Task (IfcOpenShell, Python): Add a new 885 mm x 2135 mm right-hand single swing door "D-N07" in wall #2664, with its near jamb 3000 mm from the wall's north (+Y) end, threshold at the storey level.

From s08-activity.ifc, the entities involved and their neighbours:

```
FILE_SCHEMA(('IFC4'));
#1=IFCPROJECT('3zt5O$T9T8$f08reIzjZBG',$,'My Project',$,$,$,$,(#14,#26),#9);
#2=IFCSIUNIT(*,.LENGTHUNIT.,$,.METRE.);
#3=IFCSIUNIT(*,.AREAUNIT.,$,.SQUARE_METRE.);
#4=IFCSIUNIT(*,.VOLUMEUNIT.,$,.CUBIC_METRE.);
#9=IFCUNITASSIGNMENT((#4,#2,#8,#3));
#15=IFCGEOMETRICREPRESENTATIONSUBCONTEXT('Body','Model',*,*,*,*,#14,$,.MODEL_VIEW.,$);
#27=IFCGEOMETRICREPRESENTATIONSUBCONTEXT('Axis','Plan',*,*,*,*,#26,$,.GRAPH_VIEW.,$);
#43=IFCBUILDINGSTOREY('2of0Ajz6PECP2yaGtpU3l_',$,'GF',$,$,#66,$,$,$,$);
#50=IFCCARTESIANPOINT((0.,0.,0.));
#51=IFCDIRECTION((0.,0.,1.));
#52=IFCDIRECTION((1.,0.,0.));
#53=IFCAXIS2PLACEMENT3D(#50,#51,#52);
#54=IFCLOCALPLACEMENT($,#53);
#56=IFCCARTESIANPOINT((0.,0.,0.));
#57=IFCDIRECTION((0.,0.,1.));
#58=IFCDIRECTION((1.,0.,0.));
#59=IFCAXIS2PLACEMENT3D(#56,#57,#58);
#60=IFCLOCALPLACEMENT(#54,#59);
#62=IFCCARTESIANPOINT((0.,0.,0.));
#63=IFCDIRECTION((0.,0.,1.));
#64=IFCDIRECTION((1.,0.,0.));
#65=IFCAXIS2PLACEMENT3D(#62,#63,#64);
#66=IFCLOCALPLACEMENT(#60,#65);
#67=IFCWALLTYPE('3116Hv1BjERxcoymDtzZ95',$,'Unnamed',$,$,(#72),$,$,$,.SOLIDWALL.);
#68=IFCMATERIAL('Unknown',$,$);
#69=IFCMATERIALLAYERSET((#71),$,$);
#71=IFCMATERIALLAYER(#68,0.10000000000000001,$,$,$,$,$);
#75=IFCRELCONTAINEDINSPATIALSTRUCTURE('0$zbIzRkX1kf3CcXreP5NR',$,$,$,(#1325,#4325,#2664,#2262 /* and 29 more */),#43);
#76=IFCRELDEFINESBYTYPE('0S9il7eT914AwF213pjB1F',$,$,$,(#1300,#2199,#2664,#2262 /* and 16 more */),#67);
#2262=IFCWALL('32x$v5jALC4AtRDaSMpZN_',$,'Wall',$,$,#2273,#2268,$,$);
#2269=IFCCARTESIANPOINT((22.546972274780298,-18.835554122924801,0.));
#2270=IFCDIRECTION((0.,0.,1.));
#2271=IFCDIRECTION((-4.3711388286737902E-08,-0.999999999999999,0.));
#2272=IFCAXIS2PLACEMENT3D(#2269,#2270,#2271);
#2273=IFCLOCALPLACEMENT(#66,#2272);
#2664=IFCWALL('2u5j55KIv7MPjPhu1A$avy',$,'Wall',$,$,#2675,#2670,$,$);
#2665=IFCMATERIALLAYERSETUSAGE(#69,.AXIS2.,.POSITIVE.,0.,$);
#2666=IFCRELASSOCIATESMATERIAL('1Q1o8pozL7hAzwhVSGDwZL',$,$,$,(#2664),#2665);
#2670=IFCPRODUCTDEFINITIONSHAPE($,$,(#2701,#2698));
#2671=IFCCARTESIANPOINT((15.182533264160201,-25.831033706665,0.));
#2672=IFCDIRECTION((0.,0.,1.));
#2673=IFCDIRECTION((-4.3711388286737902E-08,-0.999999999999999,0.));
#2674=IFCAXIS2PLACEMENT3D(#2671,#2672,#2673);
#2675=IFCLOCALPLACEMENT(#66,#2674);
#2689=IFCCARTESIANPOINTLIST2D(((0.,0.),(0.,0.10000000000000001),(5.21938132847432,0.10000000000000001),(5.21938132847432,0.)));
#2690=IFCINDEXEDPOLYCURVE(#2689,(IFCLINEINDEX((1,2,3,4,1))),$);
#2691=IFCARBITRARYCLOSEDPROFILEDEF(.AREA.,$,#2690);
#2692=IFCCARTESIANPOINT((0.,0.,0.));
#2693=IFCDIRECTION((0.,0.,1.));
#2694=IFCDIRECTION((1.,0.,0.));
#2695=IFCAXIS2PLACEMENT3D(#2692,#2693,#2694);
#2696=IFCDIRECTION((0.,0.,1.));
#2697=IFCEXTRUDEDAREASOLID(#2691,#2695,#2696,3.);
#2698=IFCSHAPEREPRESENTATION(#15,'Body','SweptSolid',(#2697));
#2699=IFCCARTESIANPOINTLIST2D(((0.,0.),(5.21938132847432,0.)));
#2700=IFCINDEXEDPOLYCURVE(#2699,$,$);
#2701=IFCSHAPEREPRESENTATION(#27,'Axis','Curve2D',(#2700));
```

```python
import numpy as np
import ifcopenshell
import ifcopenshell.api.feature
import ifcopenshell.api.geometry
import ifcopenshell.api.root
import ifcopenshell.api.spatial
import ifcopenshell.geom
import ifcopenshell.util.element
import ifcopenshell.util.placement
import ifcopenshell.util.representation
import ifcopenshell.util.shape
import ifcopenshell.util.unit

model = ifcopenshell.open("s08-activity.ifc")
unit_scale = ifcopenshell.util.unit.calculate_unit_scale(model)
settings = ifcopenshell.geom.settings()


def volume(element):
    """Net volume in cubic metres, openings subtracted."""
    shape = ifcopenshell.geom.create_shape(settings, element)
    return ifcopenshell.util.shape.get_volume(shape.geometry)


wall = model.by_guid("2u5j55KIv7MPjPhu1A$avy")
storey = ifcopenshell.util.element.get_container(wall, ifc_class="IfcBuildingStorey")
context = ifcopenshell.util.representation.get_context(model, "Model", "Body", "MODEL_VIEW")
before = volume(wall)

width, height, from_end, sill = 0.885, 2.135, 3, 0.0  # metres

# The wall runs along its own X axis, and the end named is its -X end.
wall_shape = ifcopenshell.geom.create_shape(settings, wall)
x, y, z = ifcopenshell.util.shape.get_vertices(wall_shape.geometry).T
start = x.min() + from_end
face, thickness = float(y.min()), float(y.max() - y.min())
wall_matrix = ifcopenshell.util.placement.get_local_placement(wall.ObjectPlacement)
level = ifcopenshell.util.placement.get_local_placement(storey.ObjectPlacement)[2, 3]


def in_wall(x, y):
    """Placement at x, y metres in the wall's axes, at sill height."""
    matrix = wall_matrix.copy()
    matrix[:, 3] = wall_matrix @ np.array([x / unit_scale, y / unit_scale, 0.0, 1.0])
    matrix[2, 3] = level + sill / unit_scale
    return matrix


# Opening: a box that overshoots both wall faces by 50 mm.
opening = ifcopenshell.api.root.create_entity(model, ifc_class="IfcOpeningElement", predefined_type="OPENING")
box = ifcopenshell.api.geometry.add_wall_representation(
    model, context=context, length=width, height=height, thickness=thickness + 0.1
)
ifcopenshell.api.geometry.assign_representation(model, product=opening, representation=box)
ifcopenshell.api.geometry.edit_object_placement(model, product=opening, matrix=in_wall(start, face - 0.05), is_si=False)
ifcopenshell.api.feature.add_feature(model, feature=opening, element=wall)

door = ifcopenshell.api.root.create_entity(model, ifc_class="IfcDoor", name="D-N07", predefined_type="DOOR")
door.OverallWidth, door.OverallHeight = width / unit_scale, height / unit_scale
door.OperationType = "SINGLE_SWING_RIGHT"
body = ifcopenshell.api.geometry.add_door_representation(
    model,
    context=context,
    overall_width=door.OverallWidth,
    overall_height=door.OverallHeight,
    operation_type="SINGLE_SWING_RIGHT",
    lining_properties={"LiningDepth": thickness / unit_scale, "ThresholdDepth": thickness / unit_scale},
)
ifcopenshell.api.geometry.assign_representation(model, product=door, representation=body)
ifcopenshell.api.spatial.assign_container(model, products=[door], relating_structure=storey)
ifcopenshell.api.feature.add_filling(model, opening=opening, element=door)

# The lining spans the wall, so the door starts at the wall face.
ifcopenshell.api.geometry.edit_object_placement(model, product=door, matrix=in_wall(start, face), is_si=False)

after = volume(wall)

print(f"wall volume {before:.3f} -> {after:.3f} m3")

model.write("s08-activity_updated.ifc")
```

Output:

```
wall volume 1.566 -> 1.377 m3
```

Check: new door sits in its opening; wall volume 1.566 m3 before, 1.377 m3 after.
